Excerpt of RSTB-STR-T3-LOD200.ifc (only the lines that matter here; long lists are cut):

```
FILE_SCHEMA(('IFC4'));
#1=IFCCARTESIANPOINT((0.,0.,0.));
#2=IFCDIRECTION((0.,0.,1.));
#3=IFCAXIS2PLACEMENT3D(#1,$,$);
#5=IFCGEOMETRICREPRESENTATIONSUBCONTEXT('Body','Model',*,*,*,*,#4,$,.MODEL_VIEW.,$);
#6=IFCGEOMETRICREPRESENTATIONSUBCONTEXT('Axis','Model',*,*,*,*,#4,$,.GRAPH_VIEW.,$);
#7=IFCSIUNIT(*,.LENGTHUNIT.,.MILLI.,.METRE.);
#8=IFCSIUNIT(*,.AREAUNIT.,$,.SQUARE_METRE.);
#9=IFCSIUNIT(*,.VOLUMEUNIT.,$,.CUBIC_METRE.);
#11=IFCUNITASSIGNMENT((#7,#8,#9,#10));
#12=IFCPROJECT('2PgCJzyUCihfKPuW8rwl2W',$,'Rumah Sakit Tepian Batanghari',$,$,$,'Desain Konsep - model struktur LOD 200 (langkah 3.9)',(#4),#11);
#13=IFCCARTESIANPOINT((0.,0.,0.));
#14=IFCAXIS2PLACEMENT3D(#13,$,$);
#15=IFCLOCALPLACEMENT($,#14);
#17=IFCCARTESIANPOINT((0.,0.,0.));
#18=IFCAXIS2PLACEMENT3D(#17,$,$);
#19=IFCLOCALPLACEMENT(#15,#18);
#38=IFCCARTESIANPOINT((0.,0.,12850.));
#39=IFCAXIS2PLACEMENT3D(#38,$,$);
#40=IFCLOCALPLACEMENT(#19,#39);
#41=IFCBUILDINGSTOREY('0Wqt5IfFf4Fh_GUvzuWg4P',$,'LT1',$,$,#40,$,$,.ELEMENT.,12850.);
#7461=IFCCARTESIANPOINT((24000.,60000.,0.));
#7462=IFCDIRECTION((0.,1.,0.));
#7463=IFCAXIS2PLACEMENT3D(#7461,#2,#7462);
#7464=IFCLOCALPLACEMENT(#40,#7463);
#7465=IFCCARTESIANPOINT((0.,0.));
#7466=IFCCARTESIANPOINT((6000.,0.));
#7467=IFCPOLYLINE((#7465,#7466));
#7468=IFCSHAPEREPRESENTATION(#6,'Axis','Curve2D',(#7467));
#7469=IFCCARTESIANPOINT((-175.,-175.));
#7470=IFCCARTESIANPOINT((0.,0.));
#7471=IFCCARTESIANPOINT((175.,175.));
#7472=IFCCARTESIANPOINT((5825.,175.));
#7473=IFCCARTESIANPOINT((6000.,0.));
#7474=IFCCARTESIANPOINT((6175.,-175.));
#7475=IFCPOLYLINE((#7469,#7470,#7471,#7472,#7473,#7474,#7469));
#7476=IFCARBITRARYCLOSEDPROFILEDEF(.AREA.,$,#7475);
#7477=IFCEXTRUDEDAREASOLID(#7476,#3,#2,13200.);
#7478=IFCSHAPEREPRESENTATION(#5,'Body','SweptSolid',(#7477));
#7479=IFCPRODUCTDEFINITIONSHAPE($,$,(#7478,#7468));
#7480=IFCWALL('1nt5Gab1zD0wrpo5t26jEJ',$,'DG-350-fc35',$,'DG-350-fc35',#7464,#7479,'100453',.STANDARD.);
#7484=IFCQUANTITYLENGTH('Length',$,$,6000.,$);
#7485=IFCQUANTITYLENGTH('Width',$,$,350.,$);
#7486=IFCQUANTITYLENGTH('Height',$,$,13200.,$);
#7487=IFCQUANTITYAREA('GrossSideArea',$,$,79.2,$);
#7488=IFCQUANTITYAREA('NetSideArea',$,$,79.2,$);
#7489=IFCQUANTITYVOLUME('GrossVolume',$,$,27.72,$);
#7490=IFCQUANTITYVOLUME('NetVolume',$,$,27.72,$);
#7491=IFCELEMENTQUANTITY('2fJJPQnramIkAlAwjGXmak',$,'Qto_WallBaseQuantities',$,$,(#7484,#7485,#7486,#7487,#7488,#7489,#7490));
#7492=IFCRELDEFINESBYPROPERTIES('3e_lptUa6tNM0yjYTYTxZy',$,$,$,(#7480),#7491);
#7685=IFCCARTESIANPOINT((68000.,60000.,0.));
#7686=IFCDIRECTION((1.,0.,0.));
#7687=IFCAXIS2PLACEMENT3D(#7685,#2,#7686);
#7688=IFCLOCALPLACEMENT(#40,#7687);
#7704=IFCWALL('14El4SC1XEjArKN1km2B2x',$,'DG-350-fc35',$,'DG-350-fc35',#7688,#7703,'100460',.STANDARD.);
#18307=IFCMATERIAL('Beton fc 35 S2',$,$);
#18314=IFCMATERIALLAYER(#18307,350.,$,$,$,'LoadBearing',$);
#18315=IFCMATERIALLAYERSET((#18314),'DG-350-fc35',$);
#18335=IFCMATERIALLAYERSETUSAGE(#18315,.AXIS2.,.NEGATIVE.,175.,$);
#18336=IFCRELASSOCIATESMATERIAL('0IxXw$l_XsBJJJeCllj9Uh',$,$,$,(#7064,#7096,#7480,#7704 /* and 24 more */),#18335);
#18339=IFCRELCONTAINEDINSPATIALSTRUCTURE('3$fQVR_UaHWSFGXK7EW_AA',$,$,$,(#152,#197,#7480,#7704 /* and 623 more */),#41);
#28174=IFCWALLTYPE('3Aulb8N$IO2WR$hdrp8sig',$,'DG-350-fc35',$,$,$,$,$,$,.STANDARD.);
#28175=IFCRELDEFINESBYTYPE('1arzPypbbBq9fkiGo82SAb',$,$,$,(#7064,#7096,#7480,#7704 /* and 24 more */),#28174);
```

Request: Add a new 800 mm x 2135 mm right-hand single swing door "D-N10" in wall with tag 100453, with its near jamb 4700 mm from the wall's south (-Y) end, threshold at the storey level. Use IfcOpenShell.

```python
import numpy as np
import ifcopenshell
import ifcopenshell.api.feature
import ifcopenshell.api.geometry
import ifcopenshell.api.pset
import ifcopenshell.api.root
import ifcopenshell.api.spatial
import ifcopenshell.geom
import ifcopenshell.util.element
import ifcopenshell.util.placement
import ifcopenshell.util.representation
import ifcopenshell.util.shape
import ifcopenshell.util.unit

model = ifcopenshell.open("RSTB-STR-T3-LOD200.ifc")
unit_scale = ifcopenshell.util.unit.calculate_unit_scale(model)
area_scale = ifcopenshell.util.unit.calculate_unit_scale(model, "AREAUNIT")
volume_scale = ifcopenshell.util.unit.calculate_unit_scale(model, "VOLUMEUNIT")
settings = ifcopenshell.geom.settings()


def volume(element):
    """Net volume in cubic metres, openings subtracted."""
    shape = ifcopenshell.geom.create_shape(settings, element)
    return ifcopenshell.util.shape.get_volume(shape.geometry)


wall = model.by_guid("1nt5Gab1zD0wrpo5t26jEJ")
storey = ifcopenshell.util.element.get_container(wall, ifc_class="IfcBuildingStorey")
context = ifcopenshell.util.representation.get_context(model, "Model", "Body", "MODEL_VIEW")
before = volume(wall)

width, height, from_end, sill = 0.8, 2.135, 4.7, 0.0  # metres

# The wall runs along its own X axis, and the end named is its -X end.
wall_shape = ifcopenshell.geom.create_shape(settings, wall)
x, y, z = ifcopenshell.util.shape.get_vertices(wall_shape.geometry).T
start = x.min() + from_end
face, thickness = float(y.min()), float(y.max() - y.min())
wall_matrix = ifcopenshell.util.placement.get_local_placement(wall.ObjectPlacement)
level = ifcopenshell.util.placement.get_local_placement(storey.ObjectPlacement)[2, 3]


def in_wall(x, y):
    """Placement at x, y metres in the wall's axes, at sill height."""
    matrix = wall_matrix.copy()
    matrix[:, 3] = wall_matrix @ np.array([x / unit_scale, y / unit_scale, 0.0, 1.0])
    matrix[2, 3] = level + sill / unit_scale
    return matrix


# Opening: a box that overshoots both wall faces by 50 mm.
opening = ifcopenshell.api.root.create_entity(model, ifc_class="IfcOpeningElement", predefined_type="OPENING")
box = ifcopenshell.api.geometry.add_wall_representation(
    model, context=context, length=width, height=height, thickness=thickness + 0.1
)
ifcopenshell.api.geometry.assign_representation(model, product=opening, representation=box)
ifcopenshell.api.geometry.edit_object_placement(model, product=opening, matrix=in_wall(start, face - 0.05), is_si=False)
ifcopenshell.api.feature.add_feature(model, feature=opening, element=wall)

door = ifcopenshell.api.root.create_entity(model, ifc_class="IfcDoor", name="D-N10", predefined_type="DOOR")
door.OverallWidth, door.OverallHeight = width / unit_scale, height / unit_scale
door.OperationType = "SINGLE_SWING_RIGHT"
body = ifcopenshell.api.geometry.add_door_representation(
    model,
    context=context,
    overall_width=door.OverallWidth,
    overall_height=door.OverallHeight,
    operation_type="SINGLE_SWING_RIGHT",
    lining_properties={"LiningDepth": thickness / unit_scale, "ThresholdDepth": thickness / unit_scale},
)
ifcopenshell.api.geometry.assign_representation(model, product=door, representation=body)
ifcopenshell.api.spatial.assign_container(model, products=[door], relating_structure=storey)
ifcopenshell.api.feature.add_filling(model, opening=opening, element=door)

# The lining spans the wall, so the door starts at the wall face.
ifcopenshell.api.geometry.edit_object_placement(model, product=door, matrix=in_wall(start, face), is_si=False)

after = volume(wall)

# Update the wall's stored quantities.
qto = model.by_id(ifcopenshell.util.element.get_pset(wall, "Qto_WallBaseQuantities", should_inherit=False)["id"])
ifcopenshell.api.pset.edit_qto(model, qto=qto, properties={
    "NetSideArea": after / thickness / area_scale,
    "NetVolume": after / volume_scale,
})

print(f"wall volume {before:.3f} -> {after:.3f} m3")

model.write("RSTB-STR-T3-LOD200_edited.ifc")
```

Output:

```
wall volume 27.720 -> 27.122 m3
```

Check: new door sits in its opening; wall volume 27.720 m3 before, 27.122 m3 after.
